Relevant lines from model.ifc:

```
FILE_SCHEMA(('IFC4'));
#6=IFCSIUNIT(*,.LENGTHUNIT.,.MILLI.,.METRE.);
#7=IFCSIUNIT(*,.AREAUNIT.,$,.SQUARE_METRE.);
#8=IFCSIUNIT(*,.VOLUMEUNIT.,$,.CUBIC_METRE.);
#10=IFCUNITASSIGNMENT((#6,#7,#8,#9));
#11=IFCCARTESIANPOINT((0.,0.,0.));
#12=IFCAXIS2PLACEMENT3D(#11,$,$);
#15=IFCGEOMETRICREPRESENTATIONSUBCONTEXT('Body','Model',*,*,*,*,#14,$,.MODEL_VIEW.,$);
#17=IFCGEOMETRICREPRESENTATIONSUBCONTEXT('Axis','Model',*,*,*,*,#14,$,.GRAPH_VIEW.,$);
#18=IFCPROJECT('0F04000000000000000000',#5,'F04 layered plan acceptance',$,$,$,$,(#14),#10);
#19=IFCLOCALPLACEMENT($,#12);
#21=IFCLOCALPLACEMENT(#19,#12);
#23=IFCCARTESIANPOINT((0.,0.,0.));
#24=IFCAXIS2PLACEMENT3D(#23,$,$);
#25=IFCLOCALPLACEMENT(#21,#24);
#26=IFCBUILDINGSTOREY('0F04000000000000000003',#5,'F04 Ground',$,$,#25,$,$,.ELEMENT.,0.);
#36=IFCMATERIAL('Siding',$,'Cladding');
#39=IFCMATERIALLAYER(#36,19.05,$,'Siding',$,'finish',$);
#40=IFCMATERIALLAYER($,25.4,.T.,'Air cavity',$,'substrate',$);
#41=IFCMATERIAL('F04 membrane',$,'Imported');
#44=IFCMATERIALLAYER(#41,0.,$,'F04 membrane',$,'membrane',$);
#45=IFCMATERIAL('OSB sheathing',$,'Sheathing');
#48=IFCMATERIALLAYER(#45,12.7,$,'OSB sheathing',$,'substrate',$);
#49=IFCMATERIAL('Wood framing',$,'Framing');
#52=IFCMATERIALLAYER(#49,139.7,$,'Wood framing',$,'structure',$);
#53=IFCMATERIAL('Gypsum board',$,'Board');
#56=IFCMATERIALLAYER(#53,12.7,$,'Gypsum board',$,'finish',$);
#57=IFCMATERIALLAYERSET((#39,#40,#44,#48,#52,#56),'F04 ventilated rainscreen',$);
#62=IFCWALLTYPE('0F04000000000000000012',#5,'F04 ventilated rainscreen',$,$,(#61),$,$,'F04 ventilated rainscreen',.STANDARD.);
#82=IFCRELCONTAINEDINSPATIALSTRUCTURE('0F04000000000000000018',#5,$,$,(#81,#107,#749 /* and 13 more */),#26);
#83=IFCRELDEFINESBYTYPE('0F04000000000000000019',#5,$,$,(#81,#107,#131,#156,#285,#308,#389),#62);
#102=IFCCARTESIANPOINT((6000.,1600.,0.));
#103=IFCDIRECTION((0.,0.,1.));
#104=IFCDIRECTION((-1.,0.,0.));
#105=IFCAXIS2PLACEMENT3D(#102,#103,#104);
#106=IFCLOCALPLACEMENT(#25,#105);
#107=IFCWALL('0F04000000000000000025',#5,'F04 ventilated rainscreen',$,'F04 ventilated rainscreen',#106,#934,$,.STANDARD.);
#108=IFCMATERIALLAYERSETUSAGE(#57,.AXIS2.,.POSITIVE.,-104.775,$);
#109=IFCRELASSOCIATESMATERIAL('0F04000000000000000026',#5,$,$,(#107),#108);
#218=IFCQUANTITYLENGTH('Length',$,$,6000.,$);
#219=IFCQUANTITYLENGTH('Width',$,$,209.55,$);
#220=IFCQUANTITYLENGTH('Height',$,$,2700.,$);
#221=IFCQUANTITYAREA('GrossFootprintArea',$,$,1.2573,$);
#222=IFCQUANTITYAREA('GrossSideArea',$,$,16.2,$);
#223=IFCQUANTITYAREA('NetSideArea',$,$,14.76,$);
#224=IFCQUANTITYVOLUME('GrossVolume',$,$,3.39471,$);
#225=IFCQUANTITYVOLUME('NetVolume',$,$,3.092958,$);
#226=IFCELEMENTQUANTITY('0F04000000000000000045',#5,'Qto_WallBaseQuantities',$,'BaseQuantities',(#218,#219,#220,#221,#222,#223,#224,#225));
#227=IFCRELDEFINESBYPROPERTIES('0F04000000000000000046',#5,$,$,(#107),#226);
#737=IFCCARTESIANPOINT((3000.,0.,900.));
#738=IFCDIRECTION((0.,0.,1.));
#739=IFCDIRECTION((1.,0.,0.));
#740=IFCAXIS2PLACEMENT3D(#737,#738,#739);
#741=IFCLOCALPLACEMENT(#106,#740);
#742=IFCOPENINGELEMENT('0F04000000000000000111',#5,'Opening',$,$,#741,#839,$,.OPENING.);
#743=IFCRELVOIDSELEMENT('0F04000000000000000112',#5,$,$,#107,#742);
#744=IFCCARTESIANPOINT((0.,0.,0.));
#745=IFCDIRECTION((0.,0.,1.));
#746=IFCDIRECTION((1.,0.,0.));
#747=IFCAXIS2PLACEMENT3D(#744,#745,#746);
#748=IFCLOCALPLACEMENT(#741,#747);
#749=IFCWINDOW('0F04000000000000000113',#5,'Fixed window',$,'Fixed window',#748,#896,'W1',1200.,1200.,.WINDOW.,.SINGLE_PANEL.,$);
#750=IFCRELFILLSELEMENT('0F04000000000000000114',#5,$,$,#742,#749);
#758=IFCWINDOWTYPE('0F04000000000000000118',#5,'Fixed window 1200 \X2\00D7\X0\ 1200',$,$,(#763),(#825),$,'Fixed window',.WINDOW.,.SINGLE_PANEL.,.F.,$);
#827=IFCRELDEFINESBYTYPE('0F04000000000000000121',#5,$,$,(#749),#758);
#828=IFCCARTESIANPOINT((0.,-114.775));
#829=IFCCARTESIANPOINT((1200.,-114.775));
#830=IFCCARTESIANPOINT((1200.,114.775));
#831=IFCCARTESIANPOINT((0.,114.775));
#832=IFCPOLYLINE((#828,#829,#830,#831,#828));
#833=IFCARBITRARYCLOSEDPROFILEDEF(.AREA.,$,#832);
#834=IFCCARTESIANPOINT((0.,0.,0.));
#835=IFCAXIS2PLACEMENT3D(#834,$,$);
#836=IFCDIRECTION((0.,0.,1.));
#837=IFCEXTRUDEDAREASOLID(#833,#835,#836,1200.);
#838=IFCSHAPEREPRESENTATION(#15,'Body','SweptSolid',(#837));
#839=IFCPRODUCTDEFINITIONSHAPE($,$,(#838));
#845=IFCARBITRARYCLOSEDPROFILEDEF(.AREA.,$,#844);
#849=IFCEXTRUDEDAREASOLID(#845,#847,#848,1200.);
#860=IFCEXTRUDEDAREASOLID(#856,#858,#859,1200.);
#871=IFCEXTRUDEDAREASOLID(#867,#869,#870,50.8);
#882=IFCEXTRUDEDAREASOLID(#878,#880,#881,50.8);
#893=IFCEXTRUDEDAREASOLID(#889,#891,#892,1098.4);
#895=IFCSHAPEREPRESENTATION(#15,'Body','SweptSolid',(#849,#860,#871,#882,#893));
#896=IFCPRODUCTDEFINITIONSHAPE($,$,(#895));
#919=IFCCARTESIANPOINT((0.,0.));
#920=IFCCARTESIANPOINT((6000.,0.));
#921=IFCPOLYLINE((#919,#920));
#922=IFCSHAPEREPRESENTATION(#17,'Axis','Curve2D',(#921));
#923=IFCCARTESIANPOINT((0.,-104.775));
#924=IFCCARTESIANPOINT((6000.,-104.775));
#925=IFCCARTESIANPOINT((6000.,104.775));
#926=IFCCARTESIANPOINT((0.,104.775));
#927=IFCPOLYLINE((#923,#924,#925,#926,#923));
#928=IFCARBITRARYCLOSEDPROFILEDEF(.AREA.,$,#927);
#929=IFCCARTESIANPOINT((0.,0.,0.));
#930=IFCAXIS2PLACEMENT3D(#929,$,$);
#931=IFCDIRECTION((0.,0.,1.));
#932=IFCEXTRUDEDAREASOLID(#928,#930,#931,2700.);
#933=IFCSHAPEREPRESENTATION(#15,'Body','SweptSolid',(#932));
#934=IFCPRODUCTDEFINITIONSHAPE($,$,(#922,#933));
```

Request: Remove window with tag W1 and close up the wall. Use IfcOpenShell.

```python
import ifcopenshell
import ifcopenshell.api.feature
import ifcopenshell.api.pset
import ifcopenshell.api.root
import ifcopenshell.geom
import ifcopenshell.util.element
import ifcopenshell.util.shape
import ifcopenshell.util.unit

model = ifcopenshell.open("model.ifc")
area_scale = ifcopenshell.util.unit.calculate_unit_scale(model, "AREAUNIT")
volume_scale = ifcopenshell.util.unit.calculate_unit_scale(model, "VOLUMEUNIT")
settings = ifcopenshell.geom.settings()


def volume(element):
    """Net volume in cubic metres, openings subtracted."""
    shape = ifcopenshell.geom.create_shape(settings, element)
    return ifcopenshell.util.shape.get_volume(shape.geometry)


window = model.by_guid("0F04000000000000000113")
opening = window.FillsVoids[0].RelatingOpeningElement
wall = opening.VoidsElements[0].RelatingBuildingElement
before = volume(wall)

ifcopenshell.api.root.remove_product(model, product=window)
ifcopenshell.api.feature.remove_feature(model, feature=opening)

after = volume(wall)
thickness = 0.2096  # wall thickness in metres

# Update the wall's stored quantities.
qto = model.by_id(ifcopenshell.util.element.get_pset(wall, "Qto_WallBaseQuantities", should_inherit=False)["id"])
ifcopenshell.api.pset.edit_qto(model, qto=qto, properties={
    "NetSideArea": after / thickness / area_scale,
    "NetVolume": after / volume_scale,
})

print(f"wall volume {before:.3f} -> {after:.3f} m3")

model.write("model-out.ifc")
```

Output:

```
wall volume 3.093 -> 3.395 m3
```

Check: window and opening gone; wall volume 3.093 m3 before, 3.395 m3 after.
